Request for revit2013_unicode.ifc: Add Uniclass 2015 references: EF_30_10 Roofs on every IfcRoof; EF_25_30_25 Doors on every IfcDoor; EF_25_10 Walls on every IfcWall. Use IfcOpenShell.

First a look at what the model holds.

```python
import ifcopenshell

model = ifcopenshell.open("revit2013_unicode.ifc")
print(model.schema)
print("classifications:", [c.Name for c in model.by_type("IfcClassification")])
for ifc_class in ("IfcDoor", "IfcRoof", "IfcStair", "IfcWall", "IfcWindow"):
    print(ifc_class, len(model.by_type(ifc_class)))
```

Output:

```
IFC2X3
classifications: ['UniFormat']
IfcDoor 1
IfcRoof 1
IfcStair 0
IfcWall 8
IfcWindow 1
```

```python
import ifcopenshell
import ifcopenshell.api.classification

model = ifcopenshell.open("revit2013_unicode.ifc")

# IFC2X3 requires Source and Edition and has no link from the project to the system.
system = model.create_entity("IfcClassification", Source="NBS", Edition="2015", Name="Uniclass 2015")

codes = {
    "IfcRoof": ("EF_30_10", "Roofs"),
    "IfcDoor": ("EF_25_30_25", "Doors"),
    "IfcWall": ("EF_25_10", "Walls"),
}
for ifc_class, (code, name) in codes.items():
    products = model.by_type(ifc_class)
    ifcopenshell.api.classification.add_reference(
        model, products=products, classification=system, identification=code, name=name
    )
    print(code, len(products))

model.write("revit2013_unicode_updated.ifc")
```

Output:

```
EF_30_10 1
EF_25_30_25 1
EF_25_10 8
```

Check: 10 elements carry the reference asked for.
